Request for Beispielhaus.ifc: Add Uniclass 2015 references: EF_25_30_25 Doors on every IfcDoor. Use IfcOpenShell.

First a look at what the model holds.

```python
import ifcopenshell

model = ifcopenshell.open("Beispielhaus.ifc")
print(model.schema)
print("classifications:", [c.Name for c in model.by_type("IfcClassification")])
for ifc_class in ("IfcDoor", "IfcRoof", "IfcStair", "IfcWall", "IfcWindow"):
    print(ifc_class, len(model.by_type(ifc_class)))
```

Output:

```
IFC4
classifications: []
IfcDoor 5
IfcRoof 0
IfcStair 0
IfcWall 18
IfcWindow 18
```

```python
import ifcopenshell
import ifcopenshell.api.classification

model = ifcopenshell.open("Beispielhaus.ifc")

system = ifcopenshell.api.classification.add_classification(model, classification="Uniclass 2015")

codes = {
    "IfcDoor": ("EF_25_30_25", "Doors"),
}
for ifc_class, (code, name) in codes.items():
    products = model.by_type(ifc_class)
    ifcopenshell.api.classification.add_reference(
        model, products=products, classification=system, identification=code, name=name
    )
    print(code, len(products))

model.write("Beispielhaus_edited.ifc")
```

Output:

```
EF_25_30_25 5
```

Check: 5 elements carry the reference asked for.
